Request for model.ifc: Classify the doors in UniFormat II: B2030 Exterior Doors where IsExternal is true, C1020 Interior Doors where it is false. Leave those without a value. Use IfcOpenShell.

First a look at what the model holds.

```python
import ifcopenshell
import ifcopenshell.util.element

model = ifcopenshell.open("model.ifc")
print(model.schema)
print("classifications:", [c.Name for c in model.by_type("IfcClassification")])
values = [ifcopenshell.util.element.get_pset(e, "Pset_DoorCommon", "IsExternal") for e in model.by_type("IfcDoor")]
for value in (True, False, None):
    print("IsExternal", value, values.count(value))
```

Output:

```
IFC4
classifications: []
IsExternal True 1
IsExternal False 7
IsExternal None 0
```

```python
import ifcopenshell
import ifcopenshell.api.classification
import ifcopenshell.util.element

model = ifcopenshell.open("model.ifc")

system = ifcopenshell.api.classification.add_classification(model, classification="UniFormat II")

doors = model.by_type("IfcDoor")
external = {e: ifcopenshell.util.element.get_pset(e, "Pset_DoorCommon", "IsExternal") for e in doors}
for flag, code, name in ((True, "B2030", "Exterior Doors"), (False, "C1020", "Interior Doors")):
    products = [e for e in doors if external[e] is flag]
    ifcopenshell.api.classification.add_reference(
        model, products=products, classification=system, identification=code, name=name
    )
    print(code, len(products))

model.write("model-out.ifc")
```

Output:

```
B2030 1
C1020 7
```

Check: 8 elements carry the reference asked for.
